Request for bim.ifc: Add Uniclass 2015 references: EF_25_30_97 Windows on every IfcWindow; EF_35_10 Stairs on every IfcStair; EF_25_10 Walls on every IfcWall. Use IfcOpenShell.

First a look at what the model holds.

```python
import ifcopenshell

model = ifcopenshell.open("bim.ifc")
print(model.schema)
print("classifications:", [c.Name for c in model.by_type("IfcClassification")])
for ifc_class in ("IfcDoor", "IfcRoof", "IfcStair", "IfcWall", "IfcWindow"):
    print(ifc_class, len(model.by_type(ifc_class)))
```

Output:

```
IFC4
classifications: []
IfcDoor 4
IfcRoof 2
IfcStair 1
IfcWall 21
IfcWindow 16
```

```python
import ifcopenshell
import ifcopenshell.api.classification

model = ifcopenshell.open("bim.ifc")

system = ifcopenshell.api.classification.add_classification(model, classification="Uniclass 2015")

codes = {
    "IfcWindow": ("EF_25_30_97", "Windows"),
    "IfcStair": ("EF_35_10", "Stairs"),
    "IfcWall": ("EF_25_10", "Walls"),
}
for ifc_class, (code, name) in codes.items():
    products = model.by_type(ifc_class)
    ifcopenshell.api.classification.add_reference(
        model, products=products, classification=system, identification=code, name=name
    )
    print(code, len(products))

model.write("bim-out.ifc")
```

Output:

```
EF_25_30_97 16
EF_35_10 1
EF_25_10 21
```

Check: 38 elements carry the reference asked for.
